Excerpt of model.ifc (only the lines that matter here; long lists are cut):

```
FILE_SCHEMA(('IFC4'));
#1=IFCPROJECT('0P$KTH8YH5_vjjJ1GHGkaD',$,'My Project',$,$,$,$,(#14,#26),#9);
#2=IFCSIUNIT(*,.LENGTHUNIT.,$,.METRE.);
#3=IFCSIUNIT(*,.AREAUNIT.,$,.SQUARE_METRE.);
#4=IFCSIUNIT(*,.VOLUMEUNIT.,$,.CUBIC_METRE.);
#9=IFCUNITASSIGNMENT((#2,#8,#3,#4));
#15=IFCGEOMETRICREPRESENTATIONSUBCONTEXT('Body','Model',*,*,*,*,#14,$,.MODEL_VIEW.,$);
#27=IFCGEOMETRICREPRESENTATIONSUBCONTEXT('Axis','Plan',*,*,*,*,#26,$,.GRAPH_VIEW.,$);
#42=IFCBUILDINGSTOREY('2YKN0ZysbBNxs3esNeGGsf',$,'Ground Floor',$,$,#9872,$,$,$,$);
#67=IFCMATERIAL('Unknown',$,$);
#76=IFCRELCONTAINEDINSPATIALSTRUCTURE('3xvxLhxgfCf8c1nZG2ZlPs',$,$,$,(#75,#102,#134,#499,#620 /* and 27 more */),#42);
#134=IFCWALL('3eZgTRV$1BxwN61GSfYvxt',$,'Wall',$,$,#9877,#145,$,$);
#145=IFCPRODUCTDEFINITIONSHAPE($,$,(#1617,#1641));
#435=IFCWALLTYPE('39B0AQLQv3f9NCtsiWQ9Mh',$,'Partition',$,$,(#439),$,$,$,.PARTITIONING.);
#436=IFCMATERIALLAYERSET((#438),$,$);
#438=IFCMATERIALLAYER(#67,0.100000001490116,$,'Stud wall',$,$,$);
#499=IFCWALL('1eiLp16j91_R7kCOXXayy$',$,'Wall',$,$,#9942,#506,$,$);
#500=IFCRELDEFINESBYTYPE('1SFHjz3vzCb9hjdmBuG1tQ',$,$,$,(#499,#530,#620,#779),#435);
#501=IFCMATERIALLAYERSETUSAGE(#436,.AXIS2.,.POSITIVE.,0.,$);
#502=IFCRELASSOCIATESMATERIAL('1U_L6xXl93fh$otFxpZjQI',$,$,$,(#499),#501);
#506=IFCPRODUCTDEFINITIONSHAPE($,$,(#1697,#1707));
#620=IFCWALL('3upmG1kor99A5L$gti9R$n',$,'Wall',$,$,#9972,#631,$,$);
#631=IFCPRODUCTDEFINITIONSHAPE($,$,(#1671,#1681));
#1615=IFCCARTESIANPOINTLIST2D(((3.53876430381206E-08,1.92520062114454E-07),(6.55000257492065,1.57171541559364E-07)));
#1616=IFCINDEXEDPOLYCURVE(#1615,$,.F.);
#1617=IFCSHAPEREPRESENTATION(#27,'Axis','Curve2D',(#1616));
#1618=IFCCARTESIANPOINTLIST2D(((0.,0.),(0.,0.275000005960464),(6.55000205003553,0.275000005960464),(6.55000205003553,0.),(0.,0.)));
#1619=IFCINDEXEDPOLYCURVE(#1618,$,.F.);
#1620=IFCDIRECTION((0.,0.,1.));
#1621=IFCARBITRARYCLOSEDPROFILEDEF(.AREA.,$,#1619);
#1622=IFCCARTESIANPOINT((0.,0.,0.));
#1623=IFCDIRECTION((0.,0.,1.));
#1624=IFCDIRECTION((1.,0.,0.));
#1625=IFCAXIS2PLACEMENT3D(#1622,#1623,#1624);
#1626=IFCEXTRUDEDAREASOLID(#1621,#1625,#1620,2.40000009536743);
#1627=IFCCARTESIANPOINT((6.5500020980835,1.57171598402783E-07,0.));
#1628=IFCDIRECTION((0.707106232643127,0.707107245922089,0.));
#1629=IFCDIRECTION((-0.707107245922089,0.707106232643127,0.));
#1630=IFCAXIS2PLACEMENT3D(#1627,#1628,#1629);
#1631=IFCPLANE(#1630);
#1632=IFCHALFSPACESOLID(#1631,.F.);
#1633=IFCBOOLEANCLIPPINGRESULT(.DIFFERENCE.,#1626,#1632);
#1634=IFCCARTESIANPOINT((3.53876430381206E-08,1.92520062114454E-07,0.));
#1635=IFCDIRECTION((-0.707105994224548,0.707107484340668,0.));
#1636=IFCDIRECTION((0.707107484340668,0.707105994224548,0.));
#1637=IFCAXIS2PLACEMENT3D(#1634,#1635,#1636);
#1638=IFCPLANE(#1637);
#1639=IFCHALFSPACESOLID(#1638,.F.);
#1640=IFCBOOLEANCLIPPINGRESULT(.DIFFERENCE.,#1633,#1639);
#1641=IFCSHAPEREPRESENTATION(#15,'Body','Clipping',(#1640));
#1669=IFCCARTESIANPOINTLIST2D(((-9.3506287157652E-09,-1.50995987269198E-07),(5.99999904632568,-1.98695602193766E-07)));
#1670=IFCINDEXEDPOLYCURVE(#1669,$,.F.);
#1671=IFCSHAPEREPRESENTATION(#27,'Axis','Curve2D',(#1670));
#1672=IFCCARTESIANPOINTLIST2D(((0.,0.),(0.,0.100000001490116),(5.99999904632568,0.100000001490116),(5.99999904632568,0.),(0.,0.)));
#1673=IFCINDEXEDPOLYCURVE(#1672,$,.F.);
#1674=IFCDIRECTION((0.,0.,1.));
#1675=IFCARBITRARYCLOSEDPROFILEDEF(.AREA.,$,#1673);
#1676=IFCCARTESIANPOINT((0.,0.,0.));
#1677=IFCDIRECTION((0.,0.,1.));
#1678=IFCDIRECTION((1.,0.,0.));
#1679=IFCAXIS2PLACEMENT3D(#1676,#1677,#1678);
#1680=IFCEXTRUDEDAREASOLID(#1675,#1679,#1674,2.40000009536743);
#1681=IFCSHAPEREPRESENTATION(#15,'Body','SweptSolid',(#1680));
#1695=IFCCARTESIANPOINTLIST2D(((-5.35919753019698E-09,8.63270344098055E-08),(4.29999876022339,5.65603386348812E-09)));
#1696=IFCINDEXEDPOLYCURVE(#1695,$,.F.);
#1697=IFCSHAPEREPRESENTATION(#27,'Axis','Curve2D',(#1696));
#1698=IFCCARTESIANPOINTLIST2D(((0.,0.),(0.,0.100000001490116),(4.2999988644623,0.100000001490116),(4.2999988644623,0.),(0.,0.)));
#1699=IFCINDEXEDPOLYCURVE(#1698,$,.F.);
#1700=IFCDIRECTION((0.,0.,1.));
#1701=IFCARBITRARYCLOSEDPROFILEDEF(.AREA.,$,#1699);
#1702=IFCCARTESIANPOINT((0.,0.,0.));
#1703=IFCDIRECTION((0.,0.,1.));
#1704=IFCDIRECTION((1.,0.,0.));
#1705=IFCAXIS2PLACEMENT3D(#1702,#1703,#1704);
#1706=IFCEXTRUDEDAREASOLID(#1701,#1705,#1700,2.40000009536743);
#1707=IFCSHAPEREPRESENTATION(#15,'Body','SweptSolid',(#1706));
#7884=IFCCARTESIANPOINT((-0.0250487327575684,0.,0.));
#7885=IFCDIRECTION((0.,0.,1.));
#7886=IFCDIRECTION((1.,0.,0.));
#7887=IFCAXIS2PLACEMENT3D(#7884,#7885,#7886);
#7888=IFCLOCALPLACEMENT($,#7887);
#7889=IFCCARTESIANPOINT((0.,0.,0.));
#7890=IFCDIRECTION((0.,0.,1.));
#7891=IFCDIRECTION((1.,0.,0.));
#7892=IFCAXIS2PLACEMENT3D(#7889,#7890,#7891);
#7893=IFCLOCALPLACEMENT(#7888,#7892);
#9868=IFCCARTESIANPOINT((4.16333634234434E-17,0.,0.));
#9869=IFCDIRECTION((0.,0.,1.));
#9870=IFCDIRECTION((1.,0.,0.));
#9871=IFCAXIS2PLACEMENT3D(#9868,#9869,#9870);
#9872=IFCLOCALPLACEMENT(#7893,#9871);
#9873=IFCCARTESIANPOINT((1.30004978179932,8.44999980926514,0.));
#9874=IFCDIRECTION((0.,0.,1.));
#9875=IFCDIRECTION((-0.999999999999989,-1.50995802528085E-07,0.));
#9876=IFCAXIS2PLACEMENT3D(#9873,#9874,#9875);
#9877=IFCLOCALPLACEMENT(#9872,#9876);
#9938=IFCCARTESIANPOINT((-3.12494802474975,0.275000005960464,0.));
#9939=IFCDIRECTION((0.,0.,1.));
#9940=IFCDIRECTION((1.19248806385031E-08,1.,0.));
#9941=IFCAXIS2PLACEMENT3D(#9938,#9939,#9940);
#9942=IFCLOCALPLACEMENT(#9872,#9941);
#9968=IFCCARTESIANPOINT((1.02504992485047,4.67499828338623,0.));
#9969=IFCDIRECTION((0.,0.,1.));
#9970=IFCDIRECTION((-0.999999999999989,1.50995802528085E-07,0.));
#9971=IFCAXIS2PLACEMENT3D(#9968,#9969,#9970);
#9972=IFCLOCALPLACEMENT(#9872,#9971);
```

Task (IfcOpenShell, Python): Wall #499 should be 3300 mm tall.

```python
import ifcopenshell
import ifcopenshell.geom
import ifcopenshell.util.representation
import ifcopenshell.util.shape
import ifcopenshell.util.unit

model = ifcopenshell.open("model.ifc")
unit_scale = ifcopenshell.util.unit.calculate_unit_scale(model)
settings = ifcopenshell.geom.settings()


def volume(element):
    """Net volume in cubic metres, openings subtracted."""
    shape = ifcopenshell.geom.create_shape(settings, element)
    return ifcopenshell.util.shape.get_volume(shape.geometry)


wall = model.by_guid("1eiLp16j91_R7kCOXXayy$")
before = volume(wall)

body = ifcopenshell.util.representation.get_representation(wall, "Model", "Body")
solid = body.Items[0]
old_height = solid.Depth
solid.Depth = 3.3 / unit_scale
after = volume(wall)

print(f"height {old_height:g} -> {solid.Depth:g}, volume {before:.3f} -> {after:.3f} m3")

model.write("model_v2.ifc")
```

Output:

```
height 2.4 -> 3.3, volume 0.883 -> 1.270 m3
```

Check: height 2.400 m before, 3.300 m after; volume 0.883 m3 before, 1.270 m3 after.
